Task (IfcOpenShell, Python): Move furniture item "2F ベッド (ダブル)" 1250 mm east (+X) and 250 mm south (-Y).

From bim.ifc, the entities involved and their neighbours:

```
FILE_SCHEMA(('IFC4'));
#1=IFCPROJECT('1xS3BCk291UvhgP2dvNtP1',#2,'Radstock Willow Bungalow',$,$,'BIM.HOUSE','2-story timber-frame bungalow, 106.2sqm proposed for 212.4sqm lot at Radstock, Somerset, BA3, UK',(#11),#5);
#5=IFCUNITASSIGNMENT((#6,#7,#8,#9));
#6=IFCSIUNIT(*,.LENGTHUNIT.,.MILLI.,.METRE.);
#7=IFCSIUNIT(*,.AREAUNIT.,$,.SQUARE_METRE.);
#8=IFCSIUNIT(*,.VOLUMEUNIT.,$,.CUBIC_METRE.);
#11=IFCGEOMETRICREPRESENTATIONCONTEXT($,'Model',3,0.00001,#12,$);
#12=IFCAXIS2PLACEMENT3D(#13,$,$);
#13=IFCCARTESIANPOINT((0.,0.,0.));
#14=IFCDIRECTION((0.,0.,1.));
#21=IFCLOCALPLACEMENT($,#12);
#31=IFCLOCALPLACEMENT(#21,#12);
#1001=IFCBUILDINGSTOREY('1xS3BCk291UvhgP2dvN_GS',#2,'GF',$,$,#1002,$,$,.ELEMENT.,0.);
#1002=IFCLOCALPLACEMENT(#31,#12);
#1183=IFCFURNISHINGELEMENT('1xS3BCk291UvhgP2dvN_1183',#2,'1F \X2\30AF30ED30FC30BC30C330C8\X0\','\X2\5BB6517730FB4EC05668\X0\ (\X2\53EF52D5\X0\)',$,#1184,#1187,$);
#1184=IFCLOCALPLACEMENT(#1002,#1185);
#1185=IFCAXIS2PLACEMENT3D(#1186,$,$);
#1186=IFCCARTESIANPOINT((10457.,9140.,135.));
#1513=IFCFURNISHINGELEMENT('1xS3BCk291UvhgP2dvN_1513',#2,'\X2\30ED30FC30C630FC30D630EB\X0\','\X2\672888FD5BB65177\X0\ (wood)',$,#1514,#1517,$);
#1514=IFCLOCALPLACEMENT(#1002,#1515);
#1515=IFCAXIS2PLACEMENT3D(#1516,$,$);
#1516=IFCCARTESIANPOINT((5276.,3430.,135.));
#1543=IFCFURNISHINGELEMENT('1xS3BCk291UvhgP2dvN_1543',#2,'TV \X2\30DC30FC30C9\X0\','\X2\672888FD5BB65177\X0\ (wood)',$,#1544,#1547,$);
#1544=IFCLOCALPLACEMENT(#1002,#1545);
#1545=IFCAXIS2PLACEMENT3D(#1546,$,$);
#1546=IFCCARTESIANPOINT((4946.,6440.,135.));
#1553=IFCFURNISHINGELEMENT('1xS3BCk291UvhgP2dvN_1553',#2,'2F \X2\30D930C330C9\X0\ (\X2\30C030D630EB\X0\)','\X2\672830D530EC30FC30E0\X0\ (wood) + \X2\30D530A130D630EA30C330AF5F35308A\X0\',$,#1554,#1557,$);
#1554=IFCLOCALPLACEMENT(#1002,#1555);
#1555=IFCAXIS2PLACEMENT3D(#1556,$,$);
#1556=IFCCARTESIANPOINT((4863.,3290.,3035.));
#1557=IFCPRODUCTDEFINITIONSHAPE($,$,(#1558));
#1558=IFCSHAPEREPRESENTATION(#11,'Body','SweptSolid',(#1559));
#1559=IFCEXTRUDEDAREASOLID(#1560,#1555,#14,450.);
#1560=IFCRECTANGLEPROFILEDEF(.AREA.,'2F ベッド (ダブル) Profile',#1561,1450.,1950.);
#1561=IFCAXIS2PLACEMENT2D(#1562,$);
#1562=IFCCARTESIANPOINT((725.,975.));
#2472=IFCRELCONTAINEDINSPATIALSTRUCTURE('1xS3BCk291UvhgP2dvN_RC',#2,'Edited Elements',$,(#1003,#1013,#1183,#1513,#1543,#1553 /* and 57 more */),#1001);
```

```python
import ifcopenshell
import ifcopenshell.api.geometry
import ifcopenshell.util.placement

model = ifcopenshell.open("bim.ifc")

item = model.by_guid("1xS3BCk291UvhgP2dvN_1553")
matrix = ifcopenshell.util.placement.get_local_placement(item.ObjectPlacement)
matrix[0, 3] += 1250.0
matrix[1, 3] -= 250.0
ifcopenshell.api.geometry.edit_object_placement(model, product=item, matrix=matrix, is_si=False)

print(ifcopenshell.util.placement.get_local_placement(item.ObjectPlacement).round(3) + 0.0)

model.write("bim_rev.ifc")
```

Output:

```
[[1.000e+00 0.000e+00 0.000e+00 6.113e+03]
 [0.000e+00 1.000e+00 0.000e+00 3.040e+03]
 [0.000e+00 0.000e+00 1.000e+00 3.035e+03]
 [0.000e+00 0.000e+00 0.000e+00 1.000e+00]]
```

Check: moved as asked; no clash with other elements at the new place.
